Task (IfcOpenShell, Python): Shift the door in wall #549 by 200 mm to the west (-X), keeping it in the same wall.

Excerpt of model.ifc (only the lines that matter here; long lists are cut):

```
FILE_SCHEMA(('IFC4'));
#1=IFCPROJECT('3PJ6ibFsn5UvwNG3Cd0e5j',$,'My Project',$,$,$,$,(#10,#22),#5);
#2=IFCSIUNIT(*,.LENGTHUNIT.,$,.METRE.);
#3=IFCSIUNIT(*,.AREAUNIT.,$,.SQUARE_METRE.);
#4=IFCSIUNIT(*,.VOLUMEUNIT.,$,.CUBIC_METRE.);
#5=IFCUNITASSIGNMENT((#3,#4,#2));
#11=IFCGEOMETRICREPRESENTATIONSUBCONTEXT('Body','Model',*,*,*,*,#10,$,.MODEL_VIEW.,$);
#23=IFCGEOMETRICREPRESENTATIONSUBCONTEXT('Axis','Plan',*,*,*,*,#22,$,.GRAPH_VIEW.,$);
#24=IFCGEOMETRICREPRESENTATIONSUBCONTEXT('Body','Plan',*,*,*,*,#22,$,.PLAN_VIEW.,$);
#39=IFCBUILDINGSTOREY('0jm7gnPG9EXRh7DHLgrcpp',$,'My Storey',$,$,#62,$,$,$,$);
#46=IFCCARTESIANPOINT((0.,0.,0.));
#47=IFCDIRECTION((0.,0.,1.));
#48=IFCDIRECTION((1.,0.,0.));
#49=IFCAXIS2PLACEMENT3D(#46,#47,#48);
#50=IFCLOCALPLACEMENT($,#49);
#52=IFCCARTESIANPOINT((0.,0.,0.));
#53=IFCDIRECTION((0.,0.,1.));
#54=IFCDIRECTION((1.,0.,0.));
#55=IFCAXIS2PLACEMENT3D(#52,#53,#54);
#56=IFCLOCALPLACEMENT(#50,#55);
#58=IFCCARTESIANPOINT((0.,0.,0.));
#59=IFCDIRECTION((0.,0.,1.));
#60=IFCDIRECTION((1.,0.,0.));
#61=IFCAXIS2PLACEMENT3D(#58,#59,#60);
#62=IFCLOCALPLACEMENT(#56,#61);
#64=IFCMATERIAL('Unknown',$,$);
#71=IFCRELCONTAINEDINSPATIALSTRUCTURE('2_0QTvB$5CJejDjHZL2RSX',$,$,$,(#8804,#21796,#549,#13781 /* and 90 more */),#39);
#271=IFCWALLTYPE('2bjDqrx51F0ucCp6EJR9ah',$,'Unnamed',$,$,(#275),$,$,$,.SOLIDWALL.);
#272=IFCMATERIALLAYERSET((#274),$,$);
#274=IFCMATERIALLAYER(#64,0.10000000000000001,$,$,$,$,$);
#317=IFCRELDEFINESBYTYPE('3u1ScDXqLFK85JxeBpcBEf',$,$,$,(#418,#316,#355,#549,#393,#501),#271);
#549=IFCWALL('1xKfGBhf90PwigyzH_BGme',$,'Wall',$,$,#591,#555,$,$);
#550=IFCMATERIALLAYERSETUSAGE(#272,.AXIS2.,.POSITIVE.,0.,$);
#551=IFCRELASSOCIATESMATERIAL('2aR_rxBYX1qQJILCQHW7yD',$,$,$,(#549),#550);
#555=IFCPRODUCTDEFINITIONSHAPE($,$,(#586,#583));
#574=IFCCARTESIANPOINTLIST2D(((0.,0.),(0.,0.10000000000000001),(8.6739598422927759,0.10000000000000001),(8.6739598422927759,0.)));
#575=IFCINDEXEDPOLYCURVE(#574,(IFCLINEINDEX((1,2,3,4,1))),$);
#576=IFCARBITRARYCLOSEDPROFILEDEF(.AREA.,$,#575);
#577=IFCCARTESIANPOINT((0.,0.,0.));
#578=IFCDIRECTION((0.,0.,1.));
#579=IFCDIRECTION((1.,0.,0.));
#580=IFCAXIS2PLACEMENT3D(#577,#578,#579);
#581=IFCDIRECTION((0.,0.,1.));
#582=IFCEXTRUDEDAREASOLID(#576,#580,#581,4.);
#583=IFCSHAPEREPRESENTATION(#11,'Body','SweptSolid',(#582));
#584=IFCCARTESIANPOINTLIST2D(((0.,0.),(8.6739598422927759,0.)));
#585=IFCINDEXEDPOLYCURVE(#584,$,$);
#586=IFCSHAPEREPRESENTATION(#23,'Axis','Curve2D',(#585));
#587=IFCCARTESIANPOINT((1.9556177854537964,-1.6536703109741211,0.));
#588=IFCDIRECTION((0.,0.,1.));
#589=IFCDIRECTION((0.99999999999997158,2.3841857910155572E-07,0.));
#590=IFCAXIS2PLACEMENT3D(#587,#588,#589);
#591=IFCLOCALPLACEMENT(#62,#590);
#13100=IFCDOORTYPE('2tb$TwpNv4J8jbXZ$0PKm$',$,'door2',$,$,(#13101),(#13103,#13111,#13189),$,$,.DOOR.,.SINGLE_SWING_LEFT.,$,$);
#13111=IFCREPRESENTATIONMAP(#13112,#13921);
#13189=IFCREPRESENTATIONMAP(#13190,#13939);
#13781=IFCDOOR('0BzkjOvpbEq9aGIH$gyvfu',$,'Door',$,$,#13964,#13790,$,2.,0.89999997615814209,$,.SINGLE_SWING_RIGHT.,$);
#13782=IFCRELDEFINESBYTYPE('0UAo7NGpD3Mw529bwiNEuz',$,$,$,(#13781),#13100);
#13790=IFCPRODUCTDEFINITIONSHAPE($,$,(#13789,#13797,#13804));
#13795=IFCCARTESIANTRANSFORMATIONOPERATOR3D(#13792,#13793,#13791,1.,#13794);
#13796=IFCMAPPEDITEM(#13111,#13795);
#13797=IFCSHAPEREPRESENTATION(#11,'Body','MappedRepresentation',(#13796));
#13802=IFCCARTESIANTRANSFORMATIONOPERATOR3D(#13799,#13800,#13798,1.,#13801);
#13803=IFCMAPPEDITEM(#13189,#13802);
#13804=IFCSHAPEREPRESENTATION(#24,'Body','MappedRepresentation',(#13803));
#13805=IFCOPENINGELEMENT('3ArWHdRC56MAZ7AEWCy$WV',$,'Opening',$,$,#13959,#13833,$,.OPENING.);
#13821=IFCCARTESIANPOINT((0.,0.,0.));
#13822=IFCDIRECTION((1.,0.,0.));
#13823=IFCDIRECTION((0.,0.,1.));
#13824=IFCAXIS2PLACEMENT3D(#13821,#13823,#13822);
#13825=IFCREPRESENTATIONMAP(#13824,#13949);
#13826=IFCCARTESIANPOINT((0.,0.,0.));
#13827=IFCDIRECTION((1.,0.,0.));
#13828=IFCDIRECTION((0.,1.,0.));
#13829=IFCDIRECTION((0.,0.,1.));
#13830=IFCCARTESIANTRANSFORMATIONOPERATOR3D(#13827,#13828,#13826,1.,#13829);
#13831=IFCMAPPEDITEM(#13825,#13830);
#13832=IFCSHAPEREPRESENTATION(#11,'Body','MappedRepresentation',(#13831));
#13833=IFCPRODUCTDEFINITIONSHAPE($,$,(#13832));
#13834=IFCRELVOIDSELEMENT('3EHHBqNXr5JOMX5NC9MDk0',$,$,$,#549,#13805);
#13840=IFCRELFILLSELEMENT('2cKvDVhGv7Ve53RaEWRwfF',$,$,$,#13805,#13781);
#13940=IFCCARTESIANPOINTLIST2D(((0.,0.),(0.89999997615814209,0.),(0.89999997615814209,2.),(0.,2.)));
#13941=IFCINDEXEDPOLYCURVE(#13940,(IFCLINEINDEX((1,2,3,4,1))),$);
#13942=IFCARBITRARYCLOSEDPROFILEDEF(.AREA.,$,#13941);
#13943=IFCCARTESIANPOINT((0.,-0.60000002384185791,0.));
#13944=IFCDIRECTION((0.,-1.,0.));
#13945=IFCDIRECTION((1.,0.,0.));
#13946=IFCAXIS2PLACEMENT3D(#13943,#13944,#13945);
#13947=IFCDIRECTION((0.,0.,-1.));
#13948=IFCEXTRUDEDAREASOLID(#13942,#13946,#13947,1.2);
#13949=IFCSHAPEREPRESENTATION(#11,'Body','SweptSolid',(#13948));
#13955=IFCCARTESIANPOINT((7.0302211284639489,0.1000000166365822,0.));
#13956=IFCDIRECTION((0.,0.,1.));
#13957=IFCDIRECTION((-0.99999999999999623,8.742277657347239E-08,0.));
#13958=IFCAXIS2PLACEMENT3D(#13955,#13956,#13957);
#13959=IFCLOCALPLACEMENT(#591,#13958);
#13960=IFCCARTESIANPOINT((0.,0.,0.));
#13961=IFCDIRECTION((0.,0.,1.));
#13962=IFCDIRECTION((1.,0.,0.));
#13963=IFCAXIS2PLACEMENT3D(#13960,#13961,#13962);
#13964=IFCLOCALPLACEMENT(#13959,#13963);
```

```python
import ifcopenshell
import ifcopenshell.api.geometry
import ifcopenshell.util.placement

model = ifcopenshell.open("model.ifc")

door = model.by_id(13781)
opening = door.FillsVoids[0].RelatingOpeningElement
wall = opening.VoidsElements[0].RelatingBuildingElement

wall_matrix = ifcopenshell.util.placement.get_local_placement(wall.ObjectPlacement)
shift = wall_matrix[:3, 0] * -0.2
before = ifcopenshell.util.placement.get_local_placement(door.ObjectPlacement)[:3, 3].copy()

# The door is placed relative to its opening, so it follows when the opening moves.
matrix = ifcopenshell.util.placement.get_local_placement(opening.ObjectPlacement)
matrix[:3, 3] += shift
ifcopenshell.api.geometry.edit_object_placement(
    model, product=opening, matrix=matrix, is_si=False, should_transform_children=True
)

after = ifcopenshell.util.placement.get_local_placement(door.ObjectPlacement)[:3, 3]
print("door moved by", (after - before).round(3) + 0.0)

model.write("model_edited.ifc")
```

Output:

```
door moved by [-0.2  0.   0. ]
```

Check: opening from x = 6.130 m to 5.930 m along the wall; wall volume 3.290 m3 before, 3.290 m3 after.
